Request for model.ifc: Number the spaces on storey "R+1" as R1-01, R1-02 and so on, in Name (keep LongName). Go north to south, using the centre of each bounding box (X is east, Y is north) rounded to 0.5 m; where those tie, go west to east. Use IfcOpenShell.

First a look at what the model holds.

```python
import ifcopenshell
import ifcopenshell.util.element
import ifcopenshell.util.placement

model = ifcopenshell.open("model.ifc")
print(model.schema)
storey = next(s for s in model.by_type("IfcBuildingStorey") if s.Name == "R+1")
spaces = [e for e in ifcopenshell.util.element.get_decomposition(storey) if e.is_a("IfcSpace")]
for e in sorted(spaces, key=lambda e: e.id()):
    origin = ifcopenshell.util.placement.get_local_placement(e.ObjectPlacement)[:3, 3]
    print(e.id(), e.Name, e.LongName, origin.round(2) + 0.0, sep=" | ")
```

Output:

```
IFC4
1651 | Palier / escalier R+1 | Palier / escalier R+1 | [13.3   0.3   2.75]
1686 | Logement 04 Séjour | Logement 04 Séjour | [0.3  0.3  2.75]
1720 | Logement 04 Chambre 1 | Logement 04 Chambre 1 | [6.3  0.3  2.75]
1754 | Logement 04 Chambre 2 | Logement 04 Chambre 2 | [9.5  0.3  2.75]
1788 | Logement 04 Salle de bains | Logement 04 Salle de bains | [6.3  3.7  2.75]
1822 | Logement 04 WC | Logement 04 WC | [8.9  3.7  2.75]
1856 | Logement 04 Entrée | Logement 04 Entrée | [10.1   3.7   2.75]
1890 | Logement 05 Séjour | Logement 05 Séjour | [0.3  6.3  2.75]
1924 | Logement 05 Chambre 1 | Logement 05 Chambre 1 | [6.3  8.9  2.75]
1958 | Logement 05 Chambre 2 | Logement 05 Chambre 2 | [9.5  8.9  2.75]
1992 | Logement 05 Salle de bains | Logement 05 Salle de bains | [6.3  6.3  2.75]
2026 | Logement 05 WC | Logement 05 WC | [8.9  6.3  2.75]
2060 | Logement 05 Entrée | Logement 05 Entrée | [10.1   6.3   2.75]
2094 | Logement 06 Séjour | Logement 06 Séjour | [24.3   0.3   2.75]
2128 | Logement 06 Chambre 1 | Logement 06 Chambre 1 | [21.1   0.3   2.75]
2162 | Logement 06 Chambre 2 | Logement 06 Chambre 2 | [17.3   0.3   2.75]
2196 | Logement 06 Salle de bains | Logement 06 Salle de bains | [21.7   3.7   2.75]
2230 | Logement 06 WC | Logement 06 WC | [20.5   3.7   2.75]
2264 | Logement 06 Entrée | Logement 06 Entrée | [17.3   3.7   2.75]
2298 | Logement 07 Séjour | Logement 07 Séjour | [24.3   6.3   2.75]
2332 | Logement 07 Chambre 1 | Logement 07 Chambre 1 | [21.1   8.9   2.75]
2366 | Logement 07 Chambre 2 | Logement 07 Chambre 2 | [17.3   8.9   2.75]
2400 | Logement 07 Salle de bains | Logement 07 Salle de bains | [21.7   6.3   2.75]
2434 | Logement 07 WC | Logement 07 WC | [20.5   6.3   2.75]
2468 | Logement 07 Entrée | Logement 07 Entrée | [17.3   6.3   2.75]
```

```python
import ifcopenshell
import ifcopenshell.geom
import ifcopenshell.util.element
import ifcopenshell.util.shape

model = ifcopenshell.open("model.ifc")
settings = ifcopenshell.geom.settings()
settings.set("use-world-coords", True)


def centre(element):
    shape = ifcopenshell.geom.create_shape(settings, element)
    return ifcopenshell.util.shape.get_bbox_centroid(shape.geometry)


storey = next(s for s in model.by_type("IfcBuildingStorey") if s.Name == "R+1")
spaces = [e for e in ifcopenshell.util.element.get_decomposition(storey) if e.is_a("IfcSpace")]

# Insertion points can sit at a corner or the storey origin, so sort by the geometry (in metres).
centres = {e: centre(e) for e in spaces}
spaces.sort(key=lambda e: (-round(centres[e][1] / 0.5), centres[e][0]))

for i, e in enumerate(spaces, start=1):
    number = f"R1-{i:02d}"
    e.Name = number
    print(e.id(), number)

model.write("model_edited.ifc")
```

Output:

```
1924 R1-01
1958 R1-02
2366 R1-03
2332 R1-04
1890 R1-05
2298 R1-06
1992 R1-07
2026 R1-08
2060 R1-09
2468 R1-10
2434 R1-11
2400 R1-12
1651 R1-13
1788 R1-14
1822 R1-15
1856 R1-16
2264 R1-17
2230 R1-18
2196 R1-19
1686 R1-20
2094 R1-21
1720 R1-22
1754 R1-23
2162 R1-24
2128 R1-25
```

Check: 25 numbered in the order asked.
